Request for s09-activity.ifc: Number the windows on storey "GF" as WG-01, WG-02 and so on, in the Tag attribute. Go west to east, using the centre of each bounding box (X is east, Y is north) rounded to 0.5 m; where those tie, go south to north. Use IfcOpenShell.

First a look at what the model holds.

```python
import ifcopenshell
import ifcopenshell.util.element
import ifcopenshell.util.placement

model = ifcopenshell.open("s09-activity.ifc")
print(model.schema)
storey = next(s for s in model.by_type("IfcBuildingStorey") if s.Name == "GF")
windows = [e for e in ifcopenshell.util.element.get_decomposition(storey) if e.is_a("IfcWindow")]
for e in sorted(windows, key=lambda e: e.id()):
    origin = ifcopenshell.util.placement.get_local_placement(e.ObjectPlacement)[:3, 3]
    print(e.id(), e.Tag, e.Name, origin.round(2) + 0.0, sep=" | ")
```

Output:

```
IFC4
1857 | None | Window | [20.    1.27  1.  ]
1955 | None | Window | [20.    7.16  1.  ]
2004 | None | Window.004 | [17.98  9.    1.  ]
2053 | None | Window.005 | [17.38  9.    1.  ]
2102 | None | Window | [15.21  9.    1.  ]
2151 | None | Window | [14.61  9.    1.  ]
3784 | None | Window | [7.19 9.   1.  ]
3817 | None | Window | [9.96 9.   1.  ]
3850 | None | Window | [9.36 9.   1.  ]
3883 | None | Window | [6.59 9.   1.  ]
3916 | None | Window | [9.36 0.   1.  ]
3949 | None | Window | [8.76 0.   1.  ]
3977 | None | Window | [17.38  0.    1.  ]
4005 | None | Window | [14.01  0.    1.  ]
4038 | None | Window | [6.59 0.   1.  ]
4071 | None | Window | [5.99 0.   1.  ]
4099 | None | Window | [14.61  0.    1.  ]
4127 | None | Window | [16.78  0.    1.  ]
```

```python
import ifcopenshell
import ifcopenshell.geom
import ifcopenshell.util.element
import ifcopenshell.util.shape

model = ifcopenshell.open("s09-activity.ifc")
settings = ifcopenshell.geom.settings()
settings.set("use-world-coords", True)


def centre(element):
    shape = ifcopenshell.geom.create_shape(settings, element)
    return ifcopenshell.util.shape.get_bbox_centroid(shape.geometry)


storey = next(s for s in model.by_type("IfcBuildingStorey") if s.Name == "GF")
windows = [e for e in ifcopenshell.util.element.get_decomposition(storey) if e.is_a("IfcWindow")]

# Insertion points can sit at a corner or the storey origin, so sort by the geometry (in metres).
centres = {e: centre(e) for e in windows}
windows.sort(key=lambda e: (round(centres[e][0] / 0.5), centres[e][1]))

for i, e in enumerate(windows, start=1):
    number = f"WG-{i:02d}"
    e.Tag = number
    print(e.id(), number)

model.write("s09-activity_rev.ifc")
```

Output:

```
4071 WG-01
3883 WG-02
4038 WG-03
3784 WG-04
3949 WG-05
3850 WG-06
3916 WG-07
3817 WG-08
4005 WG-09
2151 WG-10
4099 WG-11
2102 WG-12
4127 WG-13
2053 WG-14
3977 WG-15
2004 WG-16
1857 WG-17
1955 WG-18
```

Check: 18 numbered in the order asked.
